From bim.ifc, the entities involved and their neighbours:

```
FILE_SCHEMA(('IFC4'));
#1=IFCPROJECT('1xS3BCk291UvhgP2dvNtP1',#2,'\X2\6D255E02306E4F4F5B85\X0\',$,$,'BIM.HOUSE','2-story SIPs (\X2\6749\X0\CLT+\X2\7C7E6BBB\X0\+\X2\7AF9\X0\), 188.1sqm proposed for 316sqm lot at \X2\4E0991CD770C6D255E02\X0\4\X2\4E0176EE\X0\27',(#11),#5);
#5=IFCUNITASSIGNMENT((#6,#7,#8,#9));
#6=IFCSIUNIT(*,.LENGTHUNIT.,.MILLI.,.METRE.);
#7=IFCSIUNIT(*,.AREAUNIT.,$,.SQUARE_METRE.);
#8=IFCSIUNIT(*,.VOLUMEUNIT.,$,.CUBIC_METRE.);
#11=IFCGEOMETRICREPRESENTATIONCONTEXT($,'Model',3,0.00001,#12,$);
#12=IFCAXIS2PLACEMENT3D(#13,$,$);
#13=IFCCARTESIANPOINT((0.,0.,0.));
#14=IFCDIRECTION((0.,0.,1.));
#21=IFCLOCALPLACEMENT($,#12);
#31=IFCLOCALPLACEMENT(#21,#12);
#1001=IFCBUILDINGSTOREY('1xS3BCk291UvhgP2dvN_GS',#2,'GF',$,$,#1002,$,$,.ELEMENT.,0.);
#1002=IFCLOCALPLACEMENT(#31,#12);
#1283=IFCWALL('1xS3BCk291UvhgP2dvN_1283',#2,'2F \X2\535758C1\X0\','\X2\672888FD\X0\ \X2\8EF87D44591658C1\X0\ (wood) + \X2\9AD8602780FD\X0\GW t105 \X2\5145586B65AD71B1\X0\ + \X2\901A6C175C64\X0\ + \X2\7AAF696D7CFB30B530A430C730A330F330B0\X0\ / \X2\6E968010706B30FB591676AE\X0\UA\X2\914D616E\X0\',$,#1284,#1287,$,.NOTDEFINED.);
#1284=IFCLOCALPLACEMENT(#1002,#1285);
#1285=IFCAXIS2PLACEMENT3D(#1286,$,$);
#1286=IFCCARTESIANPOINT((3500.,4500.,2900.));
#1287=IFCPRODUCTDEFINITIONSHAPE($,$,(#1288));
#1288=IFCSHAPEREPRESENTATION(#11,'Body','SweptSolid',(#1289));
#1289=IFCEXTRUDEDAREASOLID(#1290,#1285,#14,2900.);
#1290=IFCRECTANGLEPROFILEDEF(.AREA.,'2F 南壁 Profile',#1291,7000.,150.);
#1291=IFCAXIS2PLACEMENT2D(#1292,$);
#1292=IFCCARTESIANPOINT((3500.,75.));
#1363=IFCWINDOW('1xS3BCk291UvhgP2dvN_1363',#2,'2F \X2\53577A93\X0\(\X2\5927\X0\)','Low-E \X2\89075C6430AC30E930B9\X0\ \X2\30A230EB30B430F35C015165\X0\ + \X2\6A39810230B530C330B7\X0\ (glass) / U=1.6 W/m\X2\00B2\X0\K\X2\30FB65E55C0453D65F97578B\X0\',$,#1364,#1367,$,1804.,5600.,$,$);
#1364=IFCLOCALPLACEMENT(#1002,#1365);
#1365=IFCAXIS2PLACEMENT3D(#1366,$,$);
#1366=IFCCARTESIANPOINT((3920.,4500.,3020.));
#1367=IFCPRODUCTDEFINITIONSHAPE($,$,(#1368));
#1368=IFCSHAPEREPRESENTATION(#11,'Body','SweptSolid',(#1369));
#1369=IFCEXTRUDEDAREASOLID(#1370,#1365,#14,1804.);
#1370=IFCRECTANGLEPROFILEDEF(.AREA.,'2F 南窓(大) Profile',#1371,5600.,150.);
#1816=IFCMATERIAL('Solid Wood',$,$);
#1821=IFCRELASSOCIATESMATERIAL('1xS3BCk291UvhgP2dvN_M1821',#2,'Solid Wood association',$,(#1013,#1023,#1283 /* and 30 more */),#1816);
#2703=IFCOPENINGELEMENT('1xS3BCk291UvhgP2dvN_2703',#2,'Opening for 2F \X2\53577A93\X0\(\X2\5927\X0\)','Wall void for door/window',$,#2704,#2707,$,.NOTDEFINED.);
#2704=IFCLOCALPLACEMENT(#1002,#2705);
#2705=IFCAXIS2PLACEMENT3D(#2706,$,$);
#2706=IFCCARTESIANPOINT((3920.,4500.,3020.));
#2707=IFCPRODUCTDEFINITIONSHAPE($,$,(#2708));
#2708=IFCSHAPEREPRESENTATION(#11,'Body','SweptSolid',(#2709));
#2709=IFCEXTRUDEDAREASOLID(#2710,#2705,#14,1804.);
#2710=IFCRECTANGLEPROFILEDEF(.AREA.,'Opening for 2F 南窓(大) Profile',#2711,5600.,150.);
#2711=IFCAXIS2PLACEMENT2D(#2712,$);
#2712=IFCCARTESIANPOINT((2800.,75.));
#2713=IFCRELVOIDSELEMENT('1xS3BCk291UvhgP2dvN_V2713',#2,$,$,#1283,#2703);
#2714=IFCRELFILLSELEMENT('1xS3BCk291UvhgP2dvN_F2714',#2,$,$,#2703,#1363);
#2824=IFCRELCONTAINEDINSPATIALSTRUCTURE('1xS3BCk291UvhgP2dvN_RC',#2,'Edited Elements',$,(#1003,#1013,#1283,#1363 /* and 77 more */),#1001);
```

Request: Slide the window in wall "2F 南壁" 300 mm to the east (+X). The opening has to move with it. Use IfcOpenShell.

```python
import ifcopenshell
import ifcopenshell.api.geometry
import ifcopenshell.util.placement
import ifcopenshell.util.unit

model = ifcopenshell.open("bim.ifc")
unit_scale = ifcopenshell.util.unit.calculate_unit_scale(model)

window = model.by_guid("1xS3BCk291UvhgP2dvN_1363")
opening = window.FillsVoids[0].RelatingOpeningElement
wall = opening.VoidsElements[0].RelatingBuildingElement

wall_matrix = ifcopenshell.util.placement.get_local_placement(wall.ObjectPlacement)
shift = wall_matrix[:3, 0] * 0.3 / unit_scale
before = ifcopenshell.util.placement.get_local_placement(window.ObjectPlacement)[:3, 3].copy()

# The window is not placed relative to its opening, so move both.
for product in (opening, window):
    matrix = ifcopenshell.util.placement.get_local_placement(product.ObjectPlacement)
    matrix[:3, 3] += shift
    ifcopenshell.api.geometry.edit_object_placement(model, product=product, matrix=matrix, is_si=False)

after = ifcopenshell.util.placement.get_local_placement(window.ObjectPlacement)[:3, 3]
print("window moved by", (after - before).round(3) + 0.0)

model.write("bim-out.ifc")
```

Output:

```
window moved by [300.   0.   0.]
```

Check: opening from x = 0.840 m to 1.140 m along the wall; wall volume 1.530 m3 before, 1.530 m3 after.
